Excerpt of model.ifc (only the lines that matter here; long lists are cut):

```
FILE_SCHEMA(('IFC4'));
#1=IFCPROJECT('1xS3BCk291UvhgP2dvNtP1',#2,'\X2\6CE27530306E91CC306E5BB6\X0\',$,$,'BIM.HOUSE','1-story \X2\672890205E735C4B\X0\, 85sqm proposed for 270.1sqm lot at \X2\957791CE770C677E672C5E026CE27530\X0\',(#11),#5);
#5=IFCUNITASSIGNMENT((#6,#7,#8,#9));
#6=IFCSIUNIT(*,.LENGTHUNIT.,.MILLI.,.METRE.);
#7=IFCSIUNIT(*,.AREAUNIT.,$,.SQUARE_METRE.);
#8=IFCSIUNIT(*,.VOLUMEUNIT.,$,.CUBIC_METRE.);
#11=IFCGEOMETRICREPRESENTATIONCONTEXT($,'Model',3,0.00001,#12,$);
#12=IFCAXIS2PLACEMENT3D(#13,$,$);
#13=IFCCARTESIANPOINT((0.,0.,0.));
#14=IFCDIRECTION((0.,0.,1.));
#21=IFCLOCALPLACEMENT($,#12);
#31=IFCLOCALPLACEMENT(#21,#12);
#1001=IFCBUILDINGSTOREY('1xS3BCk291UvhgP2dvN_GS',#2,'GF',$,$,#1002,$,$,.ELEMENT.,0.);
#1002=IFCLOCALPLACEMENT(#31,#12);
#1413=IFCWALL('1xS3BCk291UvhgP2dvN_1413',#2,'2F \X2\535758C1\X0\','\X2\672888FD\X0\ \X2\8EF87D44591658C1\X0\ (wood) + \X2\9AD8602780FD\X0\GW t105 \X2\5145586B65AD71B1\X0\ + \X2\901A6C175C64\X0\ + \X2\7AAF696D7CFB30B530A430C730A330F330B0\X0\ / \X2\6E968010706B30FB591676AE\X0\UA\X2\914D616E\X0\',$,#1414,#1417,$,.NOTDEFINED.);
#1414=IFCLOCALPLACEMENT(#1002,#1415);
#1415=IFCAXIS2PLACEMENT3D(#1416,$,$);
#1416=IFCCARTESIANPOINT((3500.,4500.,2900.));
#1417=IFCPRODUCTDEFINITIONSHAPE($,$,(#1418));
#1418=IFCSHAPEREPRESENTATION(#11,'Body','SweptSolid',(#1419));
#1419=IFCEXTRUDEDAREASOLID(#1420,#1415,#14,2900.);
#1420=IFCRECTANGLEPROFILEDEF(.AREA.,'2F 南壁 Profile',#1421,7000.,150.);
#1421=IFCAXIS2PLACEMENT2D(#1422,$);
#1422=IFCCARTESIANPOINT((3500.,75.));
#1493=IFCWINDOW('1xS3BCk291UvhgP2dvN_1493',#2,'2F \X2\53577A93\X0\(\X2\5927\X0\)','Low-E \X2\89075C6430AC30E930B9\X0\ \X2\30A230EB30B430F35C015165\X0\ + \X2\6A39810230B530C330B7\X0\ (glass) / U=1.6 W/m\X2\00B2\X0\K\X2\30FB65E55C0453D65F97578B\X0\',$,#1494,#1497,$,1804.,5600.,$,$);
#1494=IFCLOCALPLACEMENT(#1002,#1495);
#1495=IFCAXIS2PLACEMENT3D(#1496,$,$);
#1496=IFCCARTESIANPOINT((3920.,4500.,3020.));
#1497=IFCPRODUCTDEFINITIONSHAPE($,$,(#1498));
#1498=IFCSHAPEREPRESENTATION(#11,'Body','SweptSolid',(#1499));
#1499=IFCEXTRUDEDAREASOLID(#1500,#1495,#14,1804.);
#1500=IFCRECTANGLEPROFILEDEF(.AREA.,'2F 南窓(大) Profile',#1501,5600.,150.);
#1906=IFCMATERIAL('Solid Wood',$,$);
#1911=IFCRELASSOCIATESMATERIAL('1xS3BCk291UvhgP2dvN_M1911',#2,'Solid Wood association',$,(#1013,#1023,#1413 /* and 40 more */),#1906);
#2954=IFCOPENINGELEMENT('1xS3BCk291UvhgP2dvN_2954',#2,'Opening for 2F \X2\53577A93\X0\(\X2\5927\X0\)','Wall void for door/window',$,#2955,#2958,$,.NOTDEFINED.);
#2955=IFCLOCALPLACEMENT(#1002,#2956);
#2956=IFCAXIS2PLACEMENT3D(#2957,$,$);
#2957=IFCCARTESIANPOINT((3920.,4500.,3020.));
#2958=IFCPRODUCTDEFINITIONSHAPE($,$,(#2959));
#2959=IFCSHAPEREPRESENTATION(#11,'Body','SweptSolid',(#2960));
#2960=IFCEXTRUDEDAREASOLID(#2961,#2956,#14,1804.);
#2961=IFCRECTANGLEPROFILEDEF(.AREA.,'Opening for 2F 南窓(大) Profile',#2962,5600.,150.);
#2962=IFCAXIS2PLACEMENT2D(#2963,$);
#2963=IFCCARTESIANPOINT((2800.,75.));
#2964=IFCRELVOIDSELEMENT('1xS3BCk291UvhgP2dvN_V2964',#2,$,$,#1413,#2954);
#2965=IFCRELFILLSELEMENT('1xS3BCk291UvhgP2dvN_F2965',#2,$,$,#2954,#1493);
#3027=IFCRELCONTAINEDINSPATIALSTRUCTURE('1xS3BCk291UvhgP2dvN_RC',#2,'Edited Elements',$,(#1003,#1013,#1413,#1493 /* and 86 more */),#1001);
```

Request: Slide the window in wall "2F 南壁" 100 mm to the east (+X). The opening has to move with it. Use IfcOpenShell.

```python
import ifcopenshell
import ifcopenshell.api.geometry
import ifcopenshell.util.placement

model = ifcopenshell.open("model.ifc")

window = model.by_id(1493)
opening = window.FillsVoids[0].RelatingOpeningElement
wall = opening.VoidsElements[0].RelatingBuildingElement

wall_matrix = ifcopenshell.util.placement.get_local_placement(wall.ObjectPlacement)
shift = wall_matrix[:3, 0] * 100.0
before = ifcopenshell.util.placement.get_local_placement(window.ObjectPlacement)[:3, 3].copy()

# The window is not placed relative to its opening, so move both.
for product in (opening, window):
    matrix = ifcopenshell.util.placement.get_local_placement(product.ObjectPlacement)
    matrix[:3, 3] += shift
    ifcopenshell.api.geometry.edit_object_placement(model, product=product, matrix=matrix, is_si=False)

after = ifcopenshell.util.placement.get_local_placement(window.ObjectPlacement)[:3, 3]
print("window moved by", (after - before).round(3) + 0.0)

model.write("model-out.ifc")
```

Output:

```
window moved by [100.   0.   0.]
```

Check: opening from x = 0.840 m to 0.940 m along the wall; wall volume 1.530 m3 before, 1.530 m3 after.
